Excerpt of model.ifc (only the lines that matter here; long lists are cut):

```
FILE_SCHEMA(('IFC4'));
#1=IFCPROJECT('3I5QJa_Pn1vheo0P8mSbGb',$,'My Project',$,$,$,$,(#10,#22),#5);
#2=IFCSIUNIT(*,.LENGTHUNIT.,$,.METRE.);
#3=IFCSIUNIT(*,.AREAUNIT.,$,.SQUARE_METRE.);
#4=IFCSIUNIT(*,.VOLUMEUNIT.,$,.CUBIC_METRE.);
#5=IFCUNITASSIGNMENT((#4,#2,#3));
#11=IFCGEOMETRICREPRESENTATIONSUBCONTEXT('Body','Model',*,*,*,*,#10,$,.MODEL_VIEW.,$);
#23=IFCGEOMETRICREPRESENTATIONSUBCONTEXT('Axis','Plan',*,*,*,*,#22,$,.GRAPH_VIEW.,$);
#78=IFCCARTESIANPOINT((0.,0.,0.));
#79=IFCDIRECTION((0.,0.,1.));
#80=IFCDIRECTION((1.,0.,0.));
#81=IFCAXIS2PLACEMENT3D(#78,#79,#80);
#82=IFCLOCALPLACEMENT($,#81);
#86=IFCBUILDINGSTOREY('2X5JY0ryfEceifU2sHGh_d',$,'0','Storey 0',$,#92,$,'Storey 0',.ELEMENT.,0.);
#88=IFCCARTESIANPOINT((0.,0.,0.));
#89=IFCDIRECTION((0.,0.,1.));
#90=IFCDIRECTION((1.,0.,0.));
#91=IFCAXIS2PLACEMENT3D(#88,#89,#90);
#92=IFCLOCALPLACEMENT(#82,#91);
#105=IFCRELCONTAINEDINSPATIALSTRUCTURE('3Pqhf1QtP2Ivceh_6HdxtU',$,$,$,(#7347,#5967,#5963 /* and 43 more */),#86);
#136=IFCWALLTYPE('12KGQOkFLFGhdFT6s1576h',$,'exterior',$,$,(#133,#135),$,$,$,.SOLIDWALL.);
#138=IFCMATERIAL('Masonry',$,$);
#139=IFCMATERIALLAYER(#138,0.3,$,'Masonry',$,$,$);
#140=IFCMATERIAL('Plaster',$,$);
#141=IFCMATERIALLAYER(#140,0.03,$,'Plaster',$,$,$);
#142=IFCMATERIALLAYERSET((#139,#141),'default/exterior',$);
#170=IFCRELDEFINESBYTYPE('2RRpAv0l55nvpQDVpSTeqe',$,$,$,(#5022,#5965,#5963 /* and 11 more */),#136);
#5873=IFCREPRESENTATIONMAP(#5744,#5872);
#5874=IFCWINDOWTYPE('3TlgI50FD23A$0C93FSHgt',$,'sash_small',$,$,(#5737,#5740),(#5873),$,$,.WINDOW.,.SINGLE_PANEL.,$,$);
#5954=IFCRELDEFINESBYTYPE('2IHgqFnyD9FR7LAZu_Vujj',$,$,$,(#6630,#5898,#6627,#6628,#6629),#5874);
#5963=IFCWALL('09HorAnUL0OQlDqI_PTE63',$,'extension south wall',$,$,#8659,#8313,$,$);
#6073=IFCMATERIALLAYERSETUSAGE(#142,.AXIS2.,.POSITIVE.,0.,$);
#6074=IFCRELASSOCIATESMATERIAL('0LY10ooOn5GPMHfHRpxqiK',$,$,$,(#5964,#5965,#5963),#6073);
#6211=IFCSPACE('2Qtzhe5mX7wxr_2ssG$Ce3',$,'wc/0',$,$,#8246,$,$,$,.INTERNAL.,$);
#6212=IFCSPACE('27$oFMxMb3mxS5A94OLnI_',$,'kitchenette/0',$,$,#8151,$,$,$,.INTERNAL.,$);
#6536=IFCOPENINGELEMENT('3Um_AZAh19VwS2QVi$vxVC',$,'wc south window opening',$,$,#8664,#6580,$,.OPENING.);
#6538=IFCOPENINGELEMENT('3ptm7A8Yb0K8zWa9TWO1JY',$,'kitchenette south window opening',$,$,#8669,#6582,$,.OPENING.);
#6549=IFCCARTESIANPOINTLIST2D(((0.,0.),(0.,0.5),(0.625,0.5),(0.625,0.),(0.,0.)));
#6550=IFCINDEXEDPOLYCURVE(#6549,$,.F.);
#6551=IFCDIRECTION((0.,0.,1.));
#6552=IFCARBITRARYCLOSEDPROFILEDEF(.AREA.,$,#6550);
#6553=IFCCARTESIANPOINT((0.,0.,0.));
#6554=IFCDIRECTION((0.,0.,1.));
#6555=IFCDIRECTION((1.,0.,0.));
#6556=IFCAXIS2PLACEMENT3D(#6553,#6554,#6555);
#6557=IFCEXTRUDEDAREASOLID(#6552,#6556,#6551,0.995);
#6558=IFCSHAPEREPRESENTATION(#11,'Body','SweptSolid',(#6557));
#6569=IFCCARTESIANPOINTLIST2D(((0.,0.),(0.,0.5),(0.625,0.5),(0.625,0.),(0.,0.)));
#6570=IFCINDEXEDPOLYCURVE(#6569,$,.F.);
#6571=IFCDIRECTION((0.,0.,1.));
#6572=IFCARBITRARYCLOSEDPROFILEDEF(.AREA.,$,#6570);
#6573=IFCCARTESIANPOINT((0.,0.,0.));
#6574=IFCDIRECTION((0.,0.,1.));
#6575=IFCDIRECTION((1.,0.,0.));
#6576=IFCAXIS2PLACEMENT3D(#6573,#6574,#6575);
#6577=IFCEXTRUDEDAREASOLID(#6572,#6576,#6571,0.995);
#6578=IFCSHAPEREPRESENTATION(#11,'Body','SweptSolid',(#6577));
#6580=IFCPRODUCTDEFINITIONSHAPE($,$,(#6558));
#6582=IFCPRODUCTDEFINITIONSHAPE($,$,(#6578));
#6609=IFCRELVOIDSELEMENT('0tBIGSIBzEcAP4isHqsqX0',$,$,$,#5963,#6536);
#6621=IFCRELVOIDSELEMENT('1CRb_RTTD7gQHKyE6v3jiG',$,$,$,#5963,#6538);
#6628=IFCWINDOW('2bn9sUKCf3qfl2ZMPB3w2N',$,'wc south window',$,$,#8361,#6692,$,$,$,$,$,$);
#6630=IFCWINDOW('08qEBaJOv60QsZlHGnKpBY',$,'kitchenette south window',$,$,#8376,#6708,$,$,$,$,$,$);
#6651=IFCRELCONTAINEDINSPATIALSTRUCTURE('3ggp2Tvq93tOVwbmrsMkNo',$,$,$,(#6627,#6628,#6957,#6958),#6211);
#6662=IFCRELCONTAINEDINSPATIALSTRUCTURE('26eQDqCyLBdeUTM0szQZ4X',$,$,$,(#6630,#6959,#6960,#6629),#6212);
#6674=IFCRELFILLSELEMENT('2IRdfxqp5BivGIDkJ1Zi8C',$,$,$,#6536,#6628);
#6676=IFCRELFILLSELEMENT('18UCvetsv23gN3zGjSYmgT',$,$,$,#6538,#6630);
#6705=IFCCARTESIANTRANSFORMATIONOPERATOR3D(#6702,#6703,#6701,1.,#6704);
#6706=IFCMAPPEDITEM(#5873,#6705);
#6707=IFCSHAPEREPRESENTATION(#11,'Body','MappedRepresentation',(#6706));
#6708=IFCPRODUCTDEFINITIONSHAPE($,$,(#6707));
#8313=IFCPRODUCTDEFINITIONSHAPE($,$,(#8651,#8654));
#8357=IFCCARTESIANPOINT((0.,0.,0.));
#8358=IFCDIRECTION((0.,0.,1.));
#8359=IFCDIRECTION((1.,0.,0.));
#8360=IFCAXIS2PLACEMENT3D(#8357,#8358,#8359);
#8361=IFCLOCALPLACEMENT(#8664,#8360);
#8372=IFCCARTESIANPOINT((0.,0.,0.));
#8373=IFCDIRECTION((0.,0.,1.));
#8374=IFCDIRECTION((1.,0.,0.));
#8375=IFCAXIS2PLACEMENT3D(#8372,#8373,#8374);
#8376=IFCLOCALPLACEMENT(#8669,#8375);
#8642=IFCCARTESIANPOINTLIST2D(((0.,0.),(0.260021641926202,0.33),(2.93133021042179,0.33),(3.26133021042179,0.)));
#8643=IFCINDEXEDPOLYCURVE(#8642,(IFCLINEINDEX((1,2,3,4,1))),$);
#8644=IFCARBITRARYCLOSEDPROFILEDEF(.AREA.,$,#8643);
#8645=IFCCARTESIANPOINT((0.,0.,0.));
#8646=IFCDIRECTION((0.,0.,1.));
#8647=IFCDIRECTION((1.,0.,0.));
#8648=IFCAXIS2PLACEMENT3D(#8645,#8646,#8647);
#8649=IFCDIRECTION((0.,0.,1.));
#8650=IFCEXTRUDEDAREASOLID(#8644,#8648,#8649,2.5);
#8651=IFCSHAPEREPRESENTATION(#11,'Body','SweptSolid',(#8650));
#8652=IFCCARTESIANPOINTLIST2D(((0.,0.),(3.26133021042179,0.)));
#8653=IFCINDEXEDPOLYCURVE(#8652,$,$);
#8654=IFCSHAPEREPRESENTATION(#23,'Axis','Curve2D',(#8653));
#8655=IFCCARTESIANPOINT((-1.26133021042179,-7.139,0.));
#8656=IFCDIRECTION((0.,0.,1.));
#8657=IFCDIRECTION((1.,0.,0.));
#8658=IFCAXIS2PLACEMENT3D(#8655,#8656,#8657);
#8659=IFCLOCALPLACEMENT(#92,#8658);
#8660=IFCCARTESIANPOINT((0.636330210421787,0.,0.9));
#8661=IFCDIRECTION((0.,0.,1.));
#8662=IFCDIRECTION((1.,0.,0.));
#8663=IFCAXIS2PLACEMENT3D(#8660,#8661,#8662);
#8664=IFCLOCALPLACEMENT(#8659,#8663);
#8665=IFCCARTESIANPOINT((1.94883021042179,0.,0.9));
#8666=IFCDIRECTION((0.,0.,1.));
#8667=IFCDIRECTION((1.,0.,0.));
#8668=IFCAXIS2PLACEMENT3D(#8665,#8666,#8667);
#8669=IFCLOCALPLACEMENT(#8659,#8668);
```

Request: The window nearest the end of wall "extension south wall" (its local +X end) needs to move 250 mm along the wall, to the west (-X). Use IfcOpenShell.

```python
import ifcopenshell
import ifcopenshell.api.geometry
import ifcopenshell.util.placement
import ifcopenshell.util.unit

model = ifcopenshell.open("model.ifc")
unit_scale = ifcopenshell.util.unit.calculate_unit_scale(model)

window = model.by_guid("08qEBaJOv60QsZlHGnKpBY")
opening = window.FillsVoids[0].RelatingOpeningElement
wall = opening.VoidsElements[0].RelatingBuildingElement

wall_matrix = ifcopenshell.util.placement.get_local_placement(wall.ObjectPlacement)
shift = wall_matrix[:3, 0] * -0.25 / unit_scale
before = ifcopenshell.util.placement.get_local_placement(window.ObjectPlacement)[:3, 3].copy()

# The window is placed relative to its opening, so it follows when the opening moves.
matrix = ifcopenshell.util.placement.get_local_placement(opening.ObjectPlacement)
matrix[:3, 3] += shift
ifcopenshell.api.geometry.edit_object_placement(
    model, product=opening, matrix=matrix, is_si=False, should_transform_children=True
)

after = ifcopenshell.util.placement.get_local_placement(window.ObjectPlacement)[:3, 3]
print("window moved by", (after - before).round(3) + 0.0)

model.write("model_edited.ifc")
```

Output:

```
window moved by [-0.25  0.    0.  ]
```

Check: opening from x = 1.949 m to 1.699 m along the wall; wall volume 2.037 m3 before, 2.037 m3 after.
